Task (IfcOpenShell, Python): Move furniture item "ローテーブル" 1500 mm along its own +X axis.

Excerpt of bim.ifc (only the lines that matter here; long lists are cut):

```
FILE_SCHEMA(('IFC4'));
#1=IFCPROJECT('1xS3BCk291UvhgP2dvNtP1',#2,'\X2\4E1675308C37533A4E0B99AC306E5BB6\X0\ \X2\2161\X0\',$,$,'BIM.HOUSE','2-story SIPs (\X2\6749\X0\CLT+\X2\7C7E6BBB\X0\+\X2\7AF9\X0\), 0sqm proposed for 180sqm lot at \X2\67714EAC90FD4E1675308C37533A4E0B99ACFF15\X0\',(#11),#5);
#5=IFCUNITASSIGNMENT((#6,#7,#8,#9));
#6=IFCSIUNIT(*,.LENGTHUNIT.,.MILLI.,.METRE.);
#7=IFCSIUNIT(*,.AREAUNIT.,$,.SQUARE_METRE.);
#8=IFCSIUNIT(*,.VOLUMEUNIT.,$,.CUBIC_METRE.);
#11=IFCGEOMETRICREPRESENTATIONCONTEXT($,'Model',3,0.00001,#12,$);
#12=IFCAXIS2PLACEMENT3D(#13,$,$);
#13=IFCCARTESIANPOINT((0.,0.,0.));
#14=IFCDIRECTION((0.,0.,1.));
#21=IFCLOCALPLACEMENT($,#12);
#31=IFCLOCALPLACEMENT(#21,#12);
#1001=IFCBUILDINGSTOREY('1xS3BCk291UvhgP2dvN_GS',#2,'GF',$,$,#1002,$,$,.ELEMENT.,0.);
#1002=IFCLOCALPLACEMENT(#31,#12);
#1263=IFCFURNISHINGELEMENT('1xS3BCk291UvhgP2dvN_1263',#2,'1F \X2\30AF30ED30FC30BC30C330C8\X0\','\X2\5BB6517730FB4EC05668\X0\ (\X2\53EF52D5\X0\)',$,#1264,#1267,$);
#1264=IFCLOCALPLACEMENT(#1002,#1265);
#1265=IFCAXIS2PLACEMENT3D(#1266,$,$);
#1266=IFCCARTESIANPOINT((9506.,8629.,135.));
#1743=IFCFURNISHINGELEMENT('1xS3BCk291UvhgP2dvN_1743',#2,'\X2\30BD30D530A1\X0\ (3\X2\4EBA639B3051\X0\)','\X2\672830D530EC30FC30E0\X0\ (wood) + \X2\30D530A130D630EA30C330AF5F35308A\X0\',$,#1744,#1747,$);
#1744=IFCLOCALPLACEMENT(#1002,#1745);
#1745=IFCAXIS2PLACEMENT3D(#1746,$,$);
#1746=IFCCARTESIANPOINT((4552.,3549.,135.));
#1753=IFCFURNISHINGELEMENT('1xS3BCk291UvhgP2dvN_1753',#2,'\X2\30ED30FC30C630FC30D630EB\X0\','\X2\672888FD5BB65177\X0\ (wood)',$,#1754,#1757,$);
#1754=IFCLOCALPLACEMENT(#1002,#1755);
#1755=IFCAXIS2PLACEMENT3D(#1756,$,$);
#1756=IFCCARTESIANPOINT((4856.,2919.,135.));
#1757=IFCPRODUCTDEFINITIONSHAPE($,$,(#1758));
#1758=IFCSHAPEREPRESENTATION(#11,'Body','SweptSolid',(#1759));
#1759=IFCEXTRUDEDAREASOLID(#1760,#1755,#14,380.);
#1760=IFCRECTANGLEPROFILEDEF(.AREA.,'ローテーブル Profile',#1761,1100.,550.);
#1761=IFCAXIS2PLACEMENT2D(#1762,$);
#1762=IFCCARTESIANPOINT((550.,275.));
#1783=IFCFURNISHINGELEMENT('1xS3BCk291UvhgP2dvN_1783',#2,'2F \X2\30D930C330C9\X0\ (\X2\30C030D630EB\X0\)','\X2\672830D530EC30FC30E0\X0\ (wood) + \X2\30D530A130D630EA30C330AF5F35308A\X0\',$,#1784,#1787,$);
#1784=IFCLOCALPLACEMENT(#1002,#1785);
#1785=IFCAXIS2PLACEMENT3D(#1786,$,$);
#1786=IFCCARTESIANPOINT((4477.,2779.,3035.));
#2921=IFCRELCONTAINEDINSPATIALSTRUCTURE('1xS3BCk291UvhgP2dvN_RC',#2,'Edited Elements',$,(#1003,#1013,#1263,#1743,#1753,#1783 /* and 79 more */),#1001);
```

```python
import ifcopenshell
import ifcopenshell.api.geometry
import ifcopenshell.util.placement
import ifcopenshell.util.unit

model = ifcopenshell.open("bim.ifc")
unit_scale = ifcopenshell.util.unit.calculate_unit_scale(model)

item = model.by_id(1753)
matrix = ifcopenshell.util.placement.get_local_placement(item.ObjectPlacement)
matrix[:3, 3] += matrix[:3, 0] * 1.5 / unit_scale
ifcopenshell.api.geometry.edit_object_placement(model, product=item, matrix=matrix, is_si=False)

print(ifcopenshell.util.placement.get_local_placement(item.ObjectPlacement).round(3) + 0.0)

model.write("bim-out.ifc")
```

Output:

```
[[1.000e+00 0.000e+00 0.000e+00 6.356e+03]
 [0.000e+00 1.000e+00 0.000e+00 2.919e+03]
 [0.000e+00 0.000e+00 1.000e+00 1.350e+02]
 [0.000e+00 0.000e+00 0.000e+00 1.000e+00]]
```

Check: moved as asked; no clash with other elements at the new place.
